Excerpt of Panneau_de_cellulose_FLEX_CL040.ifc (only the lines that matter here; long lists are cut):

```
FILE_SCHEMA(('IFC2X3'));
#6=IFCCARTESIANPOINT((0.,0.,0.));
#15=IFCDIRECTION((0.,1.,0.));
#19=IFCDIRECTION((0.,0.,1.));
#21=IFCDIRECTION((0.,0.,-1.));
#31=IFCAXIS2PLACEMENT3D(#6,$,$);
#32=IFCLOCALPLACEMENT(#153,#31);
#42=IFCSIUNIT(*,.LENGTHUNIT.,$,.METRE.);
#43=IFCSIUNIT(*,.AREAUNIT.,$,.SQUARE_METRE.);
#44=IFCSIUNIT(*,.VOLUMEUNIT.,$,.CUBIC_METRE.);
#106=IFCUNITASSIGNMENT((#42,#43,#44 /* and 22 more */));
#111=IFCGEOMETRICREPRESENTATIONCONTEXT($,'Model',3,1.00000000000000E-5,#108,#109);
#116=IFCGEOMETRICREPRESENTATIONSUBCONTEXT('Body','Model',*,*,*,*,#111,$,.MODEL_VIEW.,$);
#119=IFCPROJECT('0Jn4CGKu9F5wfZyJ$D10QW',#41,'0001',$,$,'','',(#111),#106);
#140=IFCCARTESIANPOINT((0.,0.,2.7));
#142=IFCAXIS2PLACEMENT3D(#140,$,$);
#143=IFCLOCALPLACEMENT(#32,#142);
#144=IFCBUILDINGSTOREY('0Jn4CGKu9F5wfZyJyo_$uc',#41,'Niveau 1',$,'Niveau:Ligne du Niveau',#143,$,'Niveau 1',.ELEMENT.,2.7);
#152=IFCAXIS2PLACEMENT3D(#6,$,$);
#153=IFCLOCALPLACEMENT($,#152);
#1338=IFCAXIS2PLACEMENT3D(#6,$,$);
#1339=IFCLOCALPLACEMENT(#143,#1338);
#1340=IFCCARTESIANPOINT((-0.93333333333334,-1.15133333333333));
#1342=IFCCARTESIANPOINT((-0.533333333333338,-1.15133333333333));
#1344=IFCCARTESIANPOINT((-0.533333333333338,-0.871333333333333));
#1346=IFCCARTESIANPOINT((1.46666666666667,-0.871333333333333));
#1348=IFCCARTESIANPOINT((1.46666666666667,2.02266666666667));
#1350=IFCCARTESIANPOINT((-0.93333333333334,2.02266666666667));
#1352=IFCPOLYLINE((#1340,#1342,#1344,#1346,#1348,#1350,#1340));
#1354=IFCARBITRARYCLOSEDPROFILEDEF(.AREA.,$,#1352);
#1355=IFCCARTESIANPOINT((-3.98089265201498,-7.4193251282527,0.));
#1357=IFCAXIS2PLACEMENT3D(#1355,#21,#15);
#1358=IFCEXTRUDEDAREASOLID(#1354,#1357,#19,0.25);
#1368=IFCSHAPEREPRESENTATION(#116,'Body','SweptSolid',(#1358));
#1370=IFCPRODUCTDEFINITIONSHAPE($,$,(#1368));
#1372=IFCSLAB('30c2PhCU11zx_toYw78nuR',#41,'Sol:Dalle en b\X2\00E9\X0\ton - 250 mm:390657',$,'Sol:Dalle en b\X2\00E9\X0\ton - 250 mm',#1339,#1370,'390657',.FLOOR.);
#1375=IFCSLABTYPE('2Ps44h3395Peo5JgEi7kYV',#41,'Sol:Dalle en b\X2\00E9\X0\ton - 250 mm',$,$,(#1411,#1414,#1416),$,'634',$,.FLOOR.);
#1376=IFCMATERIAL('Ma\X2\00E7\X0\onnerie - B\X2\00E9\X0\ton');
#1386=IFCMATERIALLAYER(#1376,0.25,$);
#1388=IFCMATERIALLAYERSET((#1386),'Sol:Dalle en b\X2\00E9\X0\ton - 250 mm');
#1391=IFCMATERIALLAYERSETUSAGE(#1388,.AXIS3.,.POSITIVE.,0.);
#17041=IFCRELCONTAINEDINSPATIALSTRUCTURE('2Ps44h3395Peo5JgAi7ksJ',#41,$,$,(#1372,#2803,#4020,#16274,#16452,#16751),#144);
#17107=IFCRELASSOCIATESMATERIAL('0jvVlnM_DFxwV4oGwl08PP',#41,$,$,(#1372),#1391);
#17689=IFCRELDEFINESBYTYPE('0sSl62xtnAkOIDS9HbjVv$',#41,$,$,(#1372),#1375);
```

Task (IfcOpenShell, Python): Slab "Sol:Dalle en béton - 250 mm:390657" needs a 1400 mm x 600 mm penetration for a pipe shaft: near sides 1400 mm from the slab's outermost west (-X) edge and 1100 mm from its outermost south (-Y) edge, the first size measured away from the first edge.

```python
import numpy as np
import ifcopenshell
import ifcopenshell.api.feature
import ifcopenshell.api.geometry
import ifcopenshell.api.root
import ifcopenshell.geom
import ifcopenshell.util.placement
import ifcopenshell.util.representation
import ifcopenshell.util.shape
import ifcopenshell.util.unit

model = ifcopenshell.open("Panneau_de_cellulose_FLEX_CL040.ifc")
unit_scale = ifcopenshell.util.unit.calculate_unit_scale(model)
settings = ifcopenshell.geom.settings()


def volume(element):
    """Net volume in cubic metres, openings subtracted."""
    shape = ifcopenshell.geom.create_shape(settings, element)
    return ifcopenshell.util.shape.get_volume(shape.geometry)


slab = model.by_id(1372)
before = volume(slab)

# Extent in the slab's own axes, in metres. The edges named are its -X and -Y sides.
slab_shape = ifcopenshell.geom.create_shape(settings, slab)
vertices = ifcopenshell.util.shape.get_vertices(slab_shape.geometry)
x_min, y_min, bottom = vertices.min(axis=0)
top = vertices[:, 2].max()

opening = ifcopenshell.api.root.create_entity(model, ifc_class="IfcOpeningElement", name="Pipe shaft opening")
context = ifcopenshell.util.representation.get_context(model, "Model", "Body", "MODEL_VIEW")
width, depth = 1.4, 0.6
outline = [(0.0, 0.0), (width, 0.0), (width, depth), (0.0, depth), (0.0, 0.0)]
# Overshoot both faces by 50 mm so the cut is clean.
shape = ifcopenshell.api.geometry.add_slab_representation(
    model, context=context, depth=top - bottom + 0.1, polyline=outline
)
ifcopenshell.api.geometry.assign_representation(model, product=opening, representation=shape)

matrix = ifcopenshell.util.placement.get_local_placement(slab.ObjectPlacement)
matrix[:, 3] = matrix @ np.append(np.array([x_min + 1.4, y_min + 1.1, bottom - 0.05]) / unit_scale, 1.0)
ifcopenshell.api.geometry.edit_object_placement(model, product=opening, matrix=matrix, is_si=False)
ifcopenshell.api.feature.add_feature(model, feature=opening, element=slab)

after = volume(slab)

print(f"slab volume {before:.3f} -> {after:.3f} m3")

model.write("Panneau_de_cellulose_FLEX_CL040_v2.ifc")
```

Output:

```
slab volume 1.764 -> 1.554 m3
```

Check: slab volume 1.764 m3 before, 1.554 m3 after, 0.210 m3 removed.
